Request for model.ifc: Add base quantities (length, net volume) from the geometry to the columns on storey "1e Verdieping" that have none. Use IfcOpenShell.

First a look at what the model holds.

```python
import ifcopenshell
import ifcopenshell.util.element
import ifcopenshell.util.unit

model = ifcopenshell.open("model.ifc")
print(model.schema)
for unit_type in ("LENGTHUNIT", "AREAUNIT", "VOLUMEUNIT"):
    print(unit_type, ifcopenshell.util.unit.calculate_unit_scale(model, unit_type))
storey = next(s for s in model.by_type("IfcBuildingStorey") if s.Name == "1e Verdieping")
columns = [e for e in ifcopenshell.util.element.get_decomposition(storey) if e.is_a("IfcColumn")]
for e in sorted(columns, key=lambda e: e.id()):
    print(e.id(), e.is_a(), e.Name, list(ifcopenshell.util.element.get_psets(e, qtos_only=True)), sep=" | ")
```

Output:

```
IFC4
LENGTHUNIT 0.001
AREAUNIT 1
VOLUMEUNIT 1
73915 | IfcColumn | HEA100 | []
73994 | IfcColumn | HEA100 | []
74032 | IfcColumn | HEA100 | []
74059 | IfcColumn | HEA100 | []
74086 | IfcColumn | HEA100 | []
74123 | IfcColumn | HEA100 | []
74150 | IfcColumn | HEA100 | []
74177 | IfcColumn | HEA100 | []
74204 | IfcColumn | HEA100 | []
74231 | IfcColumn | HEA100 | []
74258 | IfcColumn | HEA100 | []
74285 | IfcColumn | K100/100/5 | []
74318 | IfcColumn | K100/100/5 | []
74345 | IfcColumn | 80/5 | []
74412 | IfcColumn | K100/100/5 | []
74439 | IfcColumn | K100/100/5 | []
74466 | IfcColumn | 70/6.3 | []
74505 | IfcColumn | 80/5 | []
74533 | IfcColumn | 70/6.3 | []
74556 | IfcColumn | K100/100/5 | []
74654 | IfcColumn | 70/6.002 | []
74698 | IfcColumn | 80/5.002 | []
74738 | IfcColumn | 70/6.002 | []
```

```python
import ifcopenshell
import ifcopenshell.api.pset
import ifcopenshell.geom
import ifcopenshell.util.element
import ifcopenshell.util.shape
import ifcopenshell.util.unit

model = ifcopenshell.open("model.ifc")
unit_scale = ifcopenshell.util.unit.calculate_unit_scale(model)
volume_scale = ifcopenshell.util.unit.calculate_unit_scale(model, "VOLUMEUNIT")
settings = ifcopenshell.geom.settings()

storey = next(s for s in model.by_type("IfcBuildingStorey") if s.Name == "1e Verdieping")
columns = [e for e in ifcopenshell.util.element.get_decomposition(storey) if e.is_a("IfcColumn")]

for e in sorted(columns, key=lambda e: e.id()):
    if ifcopenshell.util.element.get_psets(e, qtos_only=True, should_inherit=False):
        continue
    # Geometry comes back in metres, in the element's own axes.
    shape = ifcopenshell.geom.create_shape(settings, e)
    values = {
        "Length": ifcopenshell.util.shape.get_z(shape.geometry) / unit_scale,
        "NetVolume": ifcopenshell.util.shape.get_volume(shape.geometry) / volume_scale,
    }
    qto = ifcopenshell.api.pset.add_qto(model, product=e, name="Qto_ColumnBaseQuantities")
    ifcopenshell.api.pset.edit_qto(model, qto=qto, properties=values)
    print(e.id(), {k: round(v, 3) for k, v in values.items()})

model.write("model_updated.ifc")
```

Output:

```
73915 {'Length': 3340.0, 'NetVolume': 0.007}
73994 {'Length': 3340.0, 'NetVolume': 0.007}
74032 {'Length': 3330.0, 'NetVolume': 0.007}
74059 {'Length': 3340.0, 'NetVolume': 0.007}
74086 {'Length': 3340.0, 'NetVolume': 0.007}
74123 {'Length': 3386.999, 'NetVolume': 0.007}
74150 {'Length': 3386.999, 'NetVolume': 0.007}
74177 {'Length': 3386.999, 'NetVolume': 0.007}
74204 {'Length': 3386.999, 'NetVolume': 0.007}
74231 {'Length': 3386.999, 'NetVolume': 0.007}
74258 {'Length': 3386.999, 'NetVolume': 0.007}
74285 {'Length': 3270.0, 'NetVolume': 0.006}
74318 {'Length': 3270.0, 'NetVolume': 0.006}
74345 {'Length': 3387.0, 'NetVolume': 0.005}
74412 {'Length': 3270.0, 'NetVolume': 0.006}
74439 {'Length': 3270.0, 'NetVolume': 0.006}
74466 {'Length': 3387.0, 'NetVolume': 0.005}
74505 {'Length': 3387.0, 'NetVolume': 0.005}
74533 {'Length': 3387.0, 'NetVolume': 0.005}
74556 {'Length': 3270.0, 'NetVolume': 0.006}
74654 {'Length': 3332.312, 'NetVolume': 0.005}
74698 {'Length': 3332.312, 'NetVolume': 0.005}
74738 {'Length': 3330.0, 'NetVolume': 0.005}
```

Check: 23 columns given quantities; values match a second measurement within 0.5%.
